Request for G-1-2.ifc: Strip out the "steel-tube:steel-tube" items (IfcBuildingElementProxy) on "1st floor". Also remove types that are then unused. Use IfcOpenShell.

First a look at what the model holds.

```python
import ifcopenshell
import ifcopenshell.util.element

model = ifcopenshell.open("G-1-2.ifc")
print(model.schema)
storey = next(s for s in model.by_type("IfcBuildingStorey") if s.Name == "1st floor")
proxies = [e for e in ifcopenshell.util.element.get_decomposition(storey) if e.is_a("IfcBuildingElementProxy")]
seen = {}
for e in proxies:
    element_type = ifcopenshell.util.element.get_type(e)
    name = element_type.Name if element_type not in (None, e) else None
    seen[name] = seen.get(name, 0) + 1
for name, count in sorted(seen.items(), key=str):
    print(count, "x", name)
```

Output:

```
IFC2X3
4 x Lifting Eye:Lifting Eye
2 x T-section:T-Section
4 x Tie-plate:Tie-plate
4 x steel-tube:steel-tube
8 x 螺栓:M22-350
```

```python
import ifcopenshell
import ifcopenshell.api.root
import ifcopenshell.util.element

model = ifcopenshell.open("G-1-2.ifc")

storey = next(s for s in model.by_type("IfcBuildingStorey") if s.Name == "1st floor")
proxies = [e for e in ifcopenshell.util.element.get_decomposition(storey) if e.is_a("IfcBuildingElementProxy")]
targets = [e for e in proxies if (t := ifcopenshell.util.element.get_type(e)) not in (None, e) and t.Name == "steel-tube:steel-tube"]
types = {ifcopenshell.util.element.get_type(e) for e in targets} - {None, *targets}

for e in targets:
    ifcopenshell.api.root.remove_product(model, product=e)
print(len(targets), "removed")

unused = [t for t in types if not ifcopenshell.util.element.get_types(t)]
for t in unused:
    ifcopenshell.api.root.remove_product(model, product=t)
print(len(unused), "unused types removed")

model.write("G-1-2_v2.ifc")
```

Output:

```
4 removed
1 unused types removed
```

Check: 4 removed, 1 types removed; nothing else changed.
